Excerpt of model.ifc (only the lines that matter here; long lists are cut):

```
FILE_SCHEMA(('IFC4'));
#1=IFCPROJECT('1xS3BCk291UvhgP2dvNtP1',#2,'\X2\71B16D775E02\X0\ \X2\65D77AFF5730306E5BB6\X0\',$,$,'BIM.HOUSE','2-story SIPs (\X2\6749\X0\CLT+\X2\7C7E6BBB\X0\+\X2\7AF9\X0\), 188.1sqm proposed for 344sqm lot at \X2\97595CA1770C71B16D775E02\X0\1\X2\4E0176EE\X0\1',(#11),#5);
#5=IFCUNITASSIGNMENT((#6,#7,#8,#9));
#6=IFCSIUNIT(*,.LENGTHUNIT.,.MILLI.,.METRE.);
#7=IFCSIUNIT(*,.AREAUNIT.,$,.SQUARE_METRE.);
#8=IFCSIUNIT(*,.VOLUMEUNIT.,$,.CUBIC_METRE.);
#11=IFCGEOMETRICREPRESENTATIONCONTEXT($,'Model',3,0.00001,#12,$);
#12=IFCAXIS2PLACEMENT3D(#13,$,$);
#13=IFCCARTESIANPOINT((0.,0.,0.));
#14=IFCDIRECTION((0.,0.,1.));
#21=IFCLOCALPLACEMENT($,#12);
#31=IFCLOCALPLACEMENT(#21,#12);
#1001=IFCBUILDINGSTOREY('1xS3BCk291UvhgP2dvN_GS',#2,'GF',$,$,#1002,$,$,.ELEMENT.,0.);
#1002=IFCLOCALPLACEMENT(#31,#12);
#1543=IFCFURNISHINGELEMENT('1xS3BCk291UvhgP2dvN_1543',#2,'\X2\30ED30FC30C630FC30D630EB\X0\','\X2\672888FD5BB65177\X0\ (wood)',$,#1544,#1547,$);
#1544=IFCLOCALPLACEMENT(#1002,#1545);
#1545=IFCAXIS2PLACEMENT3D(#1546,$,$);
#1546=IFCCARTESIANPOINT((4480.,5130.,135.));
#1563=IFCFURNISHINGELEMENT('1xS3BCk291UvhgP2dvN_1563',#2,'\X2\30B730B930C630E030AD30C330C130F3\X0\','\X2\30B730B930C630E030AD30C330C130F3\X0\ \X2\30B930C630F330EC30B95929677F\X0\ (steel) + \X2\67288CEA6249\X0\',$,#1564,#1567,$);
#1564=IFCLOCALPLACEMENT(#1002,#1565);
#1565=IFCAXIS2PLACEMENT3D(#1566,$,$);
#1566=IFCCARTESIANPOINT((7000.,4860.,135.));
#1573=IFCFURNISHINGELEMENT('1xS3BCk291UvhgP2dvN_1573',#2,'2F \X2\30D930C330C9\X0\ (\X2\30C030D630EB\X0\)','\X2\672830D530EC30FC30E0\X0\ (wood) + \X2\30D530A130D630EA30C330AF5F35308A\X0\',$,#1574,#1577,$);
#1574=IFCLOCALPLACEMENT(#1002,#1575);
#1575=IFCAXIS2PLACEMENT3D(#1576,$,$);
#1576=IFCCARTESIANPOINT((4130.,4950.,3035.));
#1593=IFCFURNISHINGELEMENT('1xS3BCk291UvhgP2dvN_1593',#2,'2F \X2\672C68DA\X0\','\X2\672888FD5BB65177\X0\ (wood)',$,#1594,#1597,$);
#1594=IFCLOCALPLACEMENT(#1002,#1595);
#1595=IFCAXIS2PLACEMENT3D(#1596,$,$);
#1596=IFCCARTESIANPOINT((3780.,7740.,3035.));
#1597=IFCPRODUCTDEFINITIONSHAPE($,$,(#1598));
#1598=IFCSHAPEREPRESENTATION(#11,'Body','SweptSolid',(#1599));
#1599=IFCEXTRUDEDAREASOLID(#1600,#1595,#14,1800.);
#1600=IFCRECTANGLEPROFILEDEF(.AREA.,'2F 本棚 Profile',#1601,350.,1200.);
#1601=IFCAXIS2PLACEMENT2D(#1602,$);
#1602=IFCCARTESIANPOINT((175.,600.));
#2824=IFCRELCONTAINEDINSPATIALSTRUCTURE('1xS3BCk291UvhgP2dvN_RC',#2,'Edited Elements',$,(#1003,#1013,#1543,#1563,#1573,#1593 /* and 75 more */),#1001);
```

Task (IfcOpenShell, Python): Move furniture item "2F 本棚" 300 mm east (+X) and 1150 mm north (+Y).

```python
import ifcopenshell
import ifcopenshell.api.geometry
import ifcopenshell.util.placement

model = ifcopenshell.open("model.ifc")

item = model.by_guid("1xS3BCk291UvhgP2dvN_1593")
matrix = ifcopenshell.util.placement.get_local_placement(item.ObjectPlacement)
matrix[0, 3] += 300.0
matrix[1, 3] += 1150.0
ifcopenshell.api.geometry.edit_object_placement(model, product=item, matrix=matrix, is_si=False)

print(ifcopenshell.util.placement.get_local_placement(item.ObjectPlacement).round(3) + 0.0)

model.write("model-out.ifc")
```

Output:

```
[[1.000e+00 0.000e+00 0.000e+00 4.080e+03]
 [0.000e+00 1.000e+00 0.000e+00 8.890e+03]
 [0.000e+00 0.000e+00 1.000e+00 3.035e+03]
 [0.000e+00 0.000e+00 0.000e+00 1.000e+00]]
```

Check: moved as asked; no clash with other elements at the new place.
